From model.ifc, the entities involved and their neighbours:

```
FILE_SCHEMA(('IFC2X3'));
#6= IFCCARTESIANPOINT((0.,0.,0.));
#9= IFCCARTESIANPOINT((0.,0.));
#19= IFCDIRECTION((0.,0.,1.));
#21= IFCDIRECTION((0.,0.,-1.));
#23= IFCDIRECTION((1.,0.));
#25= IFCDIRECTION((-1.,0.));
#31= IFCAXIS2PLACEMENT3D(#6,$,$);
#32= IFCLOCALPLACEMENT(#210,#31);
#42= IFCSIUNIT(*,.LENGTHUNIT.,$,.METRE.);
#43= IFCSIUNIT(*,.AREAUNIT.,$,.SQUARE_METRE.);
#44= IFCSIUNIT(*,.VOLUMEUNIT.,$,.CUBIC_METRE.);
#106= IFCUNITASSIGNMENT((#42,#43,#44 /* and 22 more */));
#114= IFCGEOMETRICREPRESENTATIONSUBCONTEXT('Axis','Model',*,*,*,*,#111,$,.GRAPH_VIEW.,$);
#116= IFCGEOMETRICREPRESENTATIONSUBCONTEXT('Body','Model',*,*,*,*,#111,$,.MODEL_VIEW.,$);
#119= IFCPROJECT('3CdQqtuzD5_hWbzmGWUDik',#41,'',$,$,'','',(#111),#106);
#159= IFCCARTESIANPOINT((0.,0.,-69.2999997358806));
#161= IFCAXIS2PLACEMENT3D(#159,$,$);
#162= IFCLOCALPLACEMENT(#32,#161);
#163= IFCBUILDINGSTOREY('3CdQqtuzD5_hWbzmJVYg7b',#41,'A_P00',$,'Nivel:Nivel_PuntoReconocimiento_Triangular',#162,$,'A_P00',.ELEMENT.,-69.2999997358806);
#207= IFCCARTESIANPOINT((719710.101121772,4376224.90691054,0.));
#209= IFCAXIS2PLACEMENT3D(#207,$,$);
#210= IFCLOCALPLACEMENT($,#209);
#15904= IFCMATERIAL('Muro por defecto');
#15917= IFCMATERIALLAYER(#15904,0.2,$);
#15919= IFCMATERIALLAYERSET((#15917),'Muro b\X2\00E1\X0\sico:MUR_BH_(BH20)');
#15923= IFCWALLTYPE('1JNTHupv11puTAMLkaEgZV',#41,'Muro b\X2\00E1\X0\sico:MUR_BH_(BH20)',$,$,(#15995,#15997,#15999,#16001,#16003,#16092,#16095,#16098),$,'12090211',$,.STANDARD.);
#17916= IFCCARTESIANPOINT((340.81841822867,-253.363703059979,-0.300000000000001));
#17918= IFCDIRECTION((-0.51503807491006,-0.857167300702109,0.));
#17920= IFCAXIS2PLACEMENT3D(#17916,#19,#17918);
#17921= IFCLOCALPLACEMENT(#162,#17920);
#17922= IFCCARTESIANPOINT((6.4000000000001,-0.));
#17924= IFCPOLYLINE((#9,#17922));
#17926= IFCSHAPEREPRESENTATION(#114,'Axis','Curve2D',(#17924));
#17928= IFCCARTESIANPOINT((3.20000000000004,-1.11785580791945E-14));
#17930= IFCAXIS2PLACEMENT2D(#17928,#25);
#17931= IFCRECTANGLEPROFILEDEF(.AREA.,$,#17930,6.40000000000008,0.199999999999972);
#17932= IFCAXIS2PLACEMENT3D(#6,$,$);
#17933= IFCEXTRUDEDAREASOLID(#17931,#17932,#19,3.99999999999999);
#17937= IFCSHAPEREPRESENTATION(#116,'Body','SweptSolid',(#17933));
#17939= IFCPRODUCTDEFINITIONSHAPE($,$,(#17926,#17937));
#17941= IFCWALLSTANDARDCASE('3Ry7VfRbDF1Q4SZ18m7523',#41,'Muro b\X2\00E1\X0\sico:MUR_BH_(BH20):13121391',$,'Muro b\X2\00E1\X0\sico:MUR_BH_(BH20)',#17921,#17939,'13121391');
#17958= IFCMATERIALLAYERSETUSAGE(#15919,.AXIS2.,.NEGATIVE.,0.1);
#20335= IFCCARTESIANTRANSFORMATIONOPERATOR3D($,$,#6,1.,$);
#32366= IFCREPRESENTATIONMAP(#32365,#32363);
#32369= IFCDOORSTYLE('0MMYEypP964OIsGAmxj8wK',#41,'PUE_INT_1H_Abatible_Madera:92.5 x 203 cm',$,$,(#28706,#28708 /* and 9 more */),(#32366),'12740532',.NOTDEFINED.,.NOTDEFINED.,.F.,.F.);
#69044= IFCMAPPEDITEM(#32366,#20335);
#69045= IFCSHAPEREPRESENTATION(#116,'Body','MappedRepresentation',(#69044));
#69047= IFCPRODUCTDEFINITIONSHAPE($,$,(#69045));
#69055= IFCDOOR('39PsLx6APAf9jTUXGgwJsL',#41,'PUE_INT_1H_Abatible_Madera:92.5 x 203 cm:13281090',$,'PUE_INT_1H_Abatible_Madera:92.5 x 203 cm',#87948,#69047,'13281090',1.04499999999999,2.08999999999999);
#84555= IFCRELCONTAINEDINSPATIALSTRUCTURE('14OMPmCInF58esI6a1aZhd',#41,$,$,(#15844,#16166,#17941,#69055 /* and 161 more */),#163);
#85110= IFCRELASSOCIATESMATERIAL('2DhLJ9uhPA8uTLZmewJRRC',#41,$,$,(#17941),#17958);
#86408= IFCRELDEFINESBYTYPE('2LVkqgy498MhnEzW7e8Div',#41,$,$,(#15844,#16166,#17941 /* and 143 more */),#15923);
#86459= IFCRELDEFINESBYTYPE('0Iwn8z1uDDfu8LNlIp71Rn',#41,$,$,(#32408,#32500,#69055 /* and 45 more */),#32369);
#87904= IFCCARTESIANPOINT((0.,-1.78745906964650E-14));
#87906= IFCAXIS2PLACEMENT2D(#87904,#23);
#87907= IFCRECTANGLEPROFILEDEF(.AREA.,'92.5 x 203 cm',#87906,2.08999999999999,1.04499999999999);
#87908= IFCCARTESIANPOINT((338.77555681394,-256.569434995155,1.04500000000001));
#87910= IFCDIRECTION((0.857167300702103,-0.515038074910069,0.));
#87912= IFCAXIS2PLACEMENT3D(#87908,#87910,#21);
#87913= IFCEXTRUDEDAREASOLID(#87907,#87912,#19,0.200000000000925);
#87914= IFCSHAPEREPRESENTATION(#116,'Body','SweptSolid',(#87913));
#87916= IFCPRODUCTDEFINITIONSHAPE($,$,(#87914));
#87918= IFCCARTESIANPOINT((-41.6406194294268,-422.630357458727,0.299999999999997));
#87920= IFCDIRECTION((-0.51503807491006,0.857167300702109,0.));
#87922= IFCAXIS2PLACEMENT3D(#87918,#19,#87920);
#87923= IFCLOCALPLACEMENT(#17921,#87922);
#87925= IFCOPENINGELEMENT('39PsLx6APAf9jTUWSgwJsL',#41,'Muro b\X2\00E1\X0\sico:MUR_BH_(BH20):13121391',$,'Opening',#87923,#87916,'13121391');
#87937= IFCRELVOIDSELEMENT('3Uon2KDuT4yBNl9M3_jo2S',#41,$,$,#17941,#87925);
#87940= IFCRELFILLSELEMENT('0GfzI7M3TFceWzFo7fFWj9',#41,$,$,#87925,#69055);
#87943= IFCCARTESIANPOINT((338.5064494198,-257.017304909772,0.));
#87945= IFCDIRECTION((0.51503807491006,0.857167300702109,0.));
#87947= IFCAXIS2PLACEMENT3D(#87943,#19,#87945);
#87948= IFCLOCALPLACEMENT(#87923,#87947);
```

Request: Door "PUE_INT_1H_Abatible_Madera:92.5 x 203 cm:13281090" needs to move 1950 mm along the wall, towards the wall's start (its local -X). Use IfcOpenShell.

```python
import ifcopenshell
import ifcopenshell.api.geometry
import ifcopenshell.util.placement
import ifcopenshell.util.unit

model = ifcopenshell.open("model.ifc")
unit_scale = ifcopenshell.util.unit.calculate_unit_scale(model)

door = model.by_id(69055)
opening = door.FillsVoids[0].RelatingOpeningElement
wall = opening.VoidsElements[0].RelatingBuildingElement

wall_matrix = ifcopenshell.util.placement.get_local_placement(wall.ObjectPlacement)
shift = wall_matrix[:3, 0] * -1.95 / unit_scale
before = ifcopenshell.util.placement.get_local_placement(door.ObjectPlacement)[:3, 3].copy()

# The door is placed relative to its opening, so it follows when the opening moves.
matrix = ifcopenshell.util.placement.get_local_placement(opening.ObjectPlacement)
matrix[:3, 3] += shift
ifcopenshell.api.geometry.edit_object_placement(
    model, product=opening, matrix=matrix, is_si=False, should_transform_children=True
)

after = ifcopenshell.util.placement.get_local_placement(door.ObjectPlacement)[:3, 3]
print("door moved by", (after - before).round(3) + 0.0)

model.write("model_rev.ifc")
```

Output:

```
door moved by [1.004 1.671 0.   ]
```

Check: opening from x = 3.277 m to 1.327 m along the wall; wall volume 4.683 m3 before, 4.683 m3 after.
